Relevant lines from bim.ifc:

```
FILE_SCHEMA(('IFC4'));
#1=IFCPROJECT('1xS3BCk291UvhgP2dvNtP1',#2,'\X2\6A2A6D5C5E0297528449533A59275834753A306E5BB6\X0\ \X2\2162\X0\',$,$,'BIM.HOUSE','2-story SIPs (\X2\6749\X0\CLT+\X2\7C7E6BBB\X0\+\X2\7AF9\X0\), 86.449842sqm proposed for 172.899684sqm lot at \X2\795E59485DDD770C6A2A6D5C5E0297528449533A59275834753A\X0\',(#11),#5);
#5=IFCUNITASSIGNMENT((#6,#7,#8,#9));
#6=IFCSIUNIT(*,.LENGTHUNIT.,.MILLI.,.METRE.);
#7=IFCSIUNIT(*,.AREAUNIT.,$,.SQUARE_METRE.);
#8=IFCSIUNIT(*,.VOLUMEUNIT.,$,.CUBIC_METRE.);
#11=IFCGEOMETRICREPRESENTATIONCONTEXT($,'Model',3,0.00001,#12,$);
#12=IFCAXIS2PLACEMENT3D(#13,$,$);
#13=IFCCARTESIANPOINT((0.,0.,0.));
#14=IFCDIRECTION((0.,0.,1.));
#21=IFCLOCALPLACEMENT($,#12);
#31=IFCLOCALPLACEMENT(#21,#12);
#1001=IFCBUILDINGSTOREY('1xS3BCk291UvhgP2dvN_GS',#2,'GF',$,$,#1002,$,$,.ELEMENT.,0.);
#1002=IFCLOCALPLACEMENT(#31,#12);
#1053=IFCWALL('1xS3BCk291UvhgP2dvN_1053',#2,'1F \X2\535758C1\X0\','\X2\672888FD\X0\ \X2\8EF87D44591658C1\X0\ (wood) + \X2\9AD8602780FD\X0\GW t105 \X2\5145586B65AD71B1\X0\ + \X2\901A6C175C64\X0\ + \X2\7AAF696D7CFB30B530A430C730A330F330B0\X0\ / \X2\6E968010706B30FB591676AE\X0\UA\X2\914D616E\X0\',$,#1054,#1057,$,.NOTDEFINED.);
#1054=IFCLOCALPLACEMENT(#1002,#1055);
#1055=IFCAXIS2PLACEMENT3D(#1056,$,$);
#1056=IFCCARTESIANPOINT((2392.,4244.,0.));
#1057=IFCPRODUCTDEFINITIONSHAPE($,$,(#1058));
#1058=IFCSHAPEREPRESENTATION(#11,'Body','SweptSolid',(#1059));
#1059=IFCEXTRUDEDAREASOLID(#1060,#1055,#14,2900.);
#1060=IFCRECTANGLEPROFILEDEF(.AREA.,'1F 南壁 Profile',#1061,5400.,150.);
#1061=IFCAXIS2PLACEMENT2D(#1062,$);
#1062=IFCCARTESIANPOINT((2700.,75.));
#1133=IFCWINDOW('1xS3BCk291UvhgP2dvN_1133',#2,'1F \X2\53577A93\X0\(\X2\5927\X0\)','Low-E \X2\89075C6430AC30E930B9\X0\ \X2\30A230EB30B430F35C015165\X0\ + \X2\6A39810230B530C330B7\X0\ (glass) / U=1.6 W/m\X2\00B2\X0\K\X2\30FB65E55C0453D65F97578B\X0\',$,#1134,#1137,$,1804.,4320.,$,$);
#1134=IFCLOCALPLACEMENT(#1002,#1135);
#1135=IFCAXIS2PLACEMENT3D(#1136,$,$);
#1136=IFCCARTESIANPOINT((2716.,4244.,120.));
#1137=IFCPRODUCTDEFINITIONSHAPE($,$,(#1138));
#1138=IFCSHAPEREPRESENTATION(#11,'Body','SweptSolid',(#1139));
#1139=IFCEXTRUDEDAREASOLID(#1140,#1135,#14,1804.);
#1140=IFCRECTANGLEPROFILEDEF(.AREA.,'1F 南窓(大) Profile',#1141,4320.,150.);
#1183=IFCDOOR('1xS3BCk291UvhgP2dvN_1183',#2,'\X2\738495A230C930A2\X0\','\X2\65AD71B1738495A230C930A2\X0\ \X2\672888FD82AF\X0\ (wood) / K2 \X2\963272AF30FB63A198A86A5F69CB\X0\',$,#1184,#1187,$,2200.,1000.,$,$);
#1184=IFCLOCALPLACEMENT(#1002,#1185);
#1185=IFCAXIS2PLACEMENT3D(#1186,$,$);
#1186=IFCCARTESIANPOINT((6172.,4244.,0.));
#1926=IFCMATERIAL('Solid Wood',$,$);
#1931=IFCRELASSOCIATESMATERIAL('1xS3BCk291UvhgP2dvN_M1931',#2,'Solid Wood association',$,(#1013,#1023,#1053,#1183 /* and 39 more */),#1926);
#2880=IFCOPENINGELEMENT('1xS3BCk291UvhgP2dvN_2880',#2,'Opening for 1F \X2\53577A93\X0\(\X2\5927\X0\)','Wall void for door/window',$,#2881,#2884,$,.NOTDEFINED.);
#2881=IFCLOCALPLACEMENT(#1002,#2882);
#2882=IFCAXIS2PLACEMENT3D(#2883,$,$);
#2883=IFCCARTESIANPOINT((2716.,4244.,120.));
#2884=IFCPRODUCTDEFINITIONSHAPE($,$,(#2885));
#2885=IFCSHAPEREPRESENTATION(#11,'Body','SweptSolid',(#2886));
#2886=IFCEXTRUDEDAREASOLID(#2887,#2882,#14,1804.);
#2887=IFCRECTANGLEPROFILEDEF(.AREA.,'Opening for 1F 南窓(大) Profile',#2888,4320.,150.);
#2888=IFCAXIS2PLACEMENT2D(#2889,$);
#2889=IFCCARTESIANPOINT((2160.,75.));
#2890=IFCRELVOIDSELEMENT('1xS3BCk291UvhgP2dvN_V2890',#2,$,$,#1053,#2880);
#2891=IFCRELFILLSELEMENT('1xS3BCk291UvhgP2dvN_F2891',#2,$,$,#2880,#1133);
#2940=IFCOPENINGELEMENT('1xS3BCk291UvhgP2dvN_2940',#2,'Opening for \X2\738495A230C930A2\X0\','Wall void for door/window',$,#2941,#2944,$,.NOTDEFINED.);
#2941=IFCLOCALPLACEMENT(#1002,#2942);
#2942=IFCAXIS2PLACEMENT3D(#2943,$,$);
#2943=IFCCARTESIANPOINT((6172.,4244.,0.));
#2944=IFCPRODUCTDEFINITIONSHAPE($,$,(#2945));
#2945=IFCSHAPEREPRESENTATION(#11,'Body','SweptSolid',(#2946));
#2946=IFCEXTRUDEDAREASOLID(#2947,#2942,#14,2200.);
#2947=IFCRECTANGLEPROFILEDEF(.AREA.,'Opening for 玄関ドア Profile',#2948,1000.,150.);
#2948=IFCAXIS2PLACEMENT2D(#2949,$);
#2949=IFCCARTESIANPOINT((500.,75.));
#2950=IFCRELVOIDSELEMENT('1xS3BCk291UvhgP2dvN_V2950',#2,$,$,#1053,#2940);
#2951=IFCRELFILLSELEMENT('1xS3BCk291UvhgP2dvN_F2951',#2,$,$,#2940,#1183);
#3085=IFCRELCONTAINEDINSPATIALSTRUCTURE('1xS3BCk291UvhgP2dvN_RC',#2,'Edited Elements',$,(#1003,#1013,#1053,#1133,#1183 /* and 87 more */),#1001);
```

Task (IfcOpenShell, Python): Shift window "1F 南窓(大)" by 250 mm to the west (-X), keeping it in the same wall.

```python
import ifcopenshell
import ifcopenshell.api.geometry
import ifcopenshell.util.placement

model = ifcopenshell.open("bim.ifc")

window = model.by_guid("1xS3BCk291UvhgP2dvN_1133")
opening = window.FillsVoids[0].RelatingOpeningElement
wall = opening.VoidsElements[0].RelatingBuildingElement

wall_matrix = ifcopenshell.util.placement.get_local_placement(wall.ObjectPlacement)
shift = wall_matrix[:3, 0] * -250.0
before = ifcopenshell.util.placement.get_local_placement(window.ObjectPlacement)[:3, 3].copy()

# The window is not placed relative to its opening, so move both.
for product in (opening, window):
    matrix = ifcopenshell.util.placement.get_local_placement(product.ObjectPlacement)
    matrix[:3, 3] += shift
    ifcopenshell.api.geometry.edit_object_placement(model, product=product, matrix=matrix, is_si=False)

after = ifcopenshell.util.placement.get_local_placement(window.ObjectPlacement)[:3, 3]
print("window moved by", (after - before).round(3) + 0.0)

model.write("bim_updated.ifc")
```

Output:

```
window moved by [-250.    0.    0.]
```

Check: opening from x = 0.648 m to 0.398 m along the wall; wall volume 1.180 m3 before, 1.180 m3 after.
